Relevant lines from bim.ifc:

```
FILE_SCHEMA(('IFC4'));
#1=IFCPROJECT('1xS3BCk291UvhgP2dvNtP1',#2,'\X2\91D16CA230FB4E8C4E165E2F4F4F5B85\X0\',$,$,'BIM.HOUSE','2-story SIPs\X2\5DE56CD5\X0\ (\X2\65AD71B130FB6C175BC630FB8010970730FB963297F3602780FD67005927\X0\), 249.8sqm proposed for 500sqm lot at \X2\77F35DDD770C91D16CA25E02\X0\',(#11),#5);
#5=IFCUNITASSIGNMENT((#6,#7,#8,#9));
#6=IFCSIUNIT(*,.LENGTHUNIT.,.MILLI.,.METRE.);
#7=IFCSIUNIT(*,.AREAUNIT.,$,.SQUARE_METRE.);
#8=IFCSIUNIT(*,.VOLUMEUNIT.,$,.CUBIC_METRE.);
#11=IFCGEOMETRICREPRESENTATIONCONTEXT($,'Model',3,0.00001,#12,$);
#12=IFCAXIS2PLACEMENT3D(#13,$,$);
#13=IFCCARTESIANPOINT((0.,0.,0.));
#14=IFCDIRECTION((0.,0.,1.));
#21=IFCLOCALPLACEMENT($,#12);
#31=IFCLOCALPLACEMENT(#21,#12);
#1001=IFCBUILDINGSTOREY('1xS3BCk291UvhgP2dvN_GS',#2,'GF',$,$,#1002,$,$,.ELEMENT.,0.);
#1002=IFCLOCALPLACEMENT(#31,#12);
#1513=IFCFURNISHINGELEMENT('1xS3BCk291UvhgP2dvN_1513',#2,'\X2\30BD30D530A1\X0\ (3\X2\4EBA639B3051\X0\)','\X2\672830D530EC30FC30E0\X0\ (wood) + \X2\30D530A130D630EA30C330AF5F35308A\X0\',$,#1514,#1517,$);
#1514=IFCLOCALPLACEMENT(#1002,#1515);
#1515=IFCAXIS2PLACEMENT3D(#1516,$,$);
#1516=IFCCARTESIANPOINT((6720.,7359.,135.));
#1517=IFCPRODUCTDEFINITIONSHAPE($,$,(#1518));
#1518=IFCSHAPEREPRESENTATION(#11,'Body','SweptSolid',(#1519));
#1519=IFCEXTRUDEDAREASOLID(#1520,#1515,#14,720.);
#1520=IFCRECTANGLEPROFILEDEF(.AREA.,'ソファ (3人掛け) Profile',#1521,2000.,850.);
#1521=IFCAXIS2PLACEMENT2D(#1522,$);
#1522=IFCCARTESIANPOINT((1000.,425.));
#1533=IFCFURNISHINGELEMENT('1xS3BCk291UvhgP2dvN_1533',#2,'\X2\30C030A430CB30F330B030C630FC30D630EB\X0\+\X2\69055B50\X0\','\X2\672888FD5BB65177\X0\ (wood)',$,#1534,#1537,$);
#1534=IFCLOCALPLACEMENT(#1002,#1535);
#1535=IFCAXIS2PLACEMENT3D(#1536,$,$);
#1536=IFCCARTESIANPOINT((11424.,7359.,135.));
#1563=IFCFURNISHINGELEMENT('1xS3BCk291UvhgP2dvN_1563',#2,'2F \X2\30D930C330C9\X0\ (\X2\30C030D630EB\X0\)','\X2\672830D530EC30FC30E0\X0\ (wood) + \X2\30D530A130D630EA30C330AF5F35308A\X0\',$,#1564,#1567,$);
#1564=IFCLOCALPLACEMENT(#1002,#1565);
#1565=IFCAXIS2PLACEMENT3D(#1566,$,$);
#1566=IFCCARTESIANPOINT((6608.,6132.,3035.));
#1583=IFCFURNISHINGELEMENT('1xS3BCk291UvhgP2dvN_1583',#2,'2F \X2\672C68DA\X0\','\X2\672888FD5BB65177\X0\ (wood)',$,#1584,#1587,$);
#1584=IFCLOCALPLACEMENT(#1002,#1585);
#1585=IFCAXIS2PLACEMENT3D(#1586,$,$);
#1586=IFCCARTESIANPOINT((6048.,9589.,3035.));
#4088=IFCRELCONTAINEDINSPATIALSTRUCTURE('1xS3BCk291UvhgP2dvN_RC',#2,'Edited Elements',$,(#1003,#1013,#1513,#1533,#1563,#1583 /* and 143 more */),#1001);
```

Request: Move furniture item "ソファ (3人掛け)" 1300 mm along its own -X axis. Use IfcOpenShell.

```python
import ifcopenshell
import ifcopenshell.api.geometry
import ifcopenshell.util.placement

model = ifcopenshell.open("bim.ifc")

item = model.by_guid("1xS3BCk291UvhgP2dvN_1513")
matrix = ifcopenshell.util.placement.get_local_placement(item.ObjectPlacement)
matrix[:3, 3] -= matrix[:3, 0] * 1300.0
ifcopenshell.api.geometry.edit_object_placement(model, product=item, matrix=matrix, is_si=False)

print(ifcopenshell.util.placement.get_local_placement(item.ObjectPlacement).round(3) + 0.0)

model.write("bim_updated.ifc")
```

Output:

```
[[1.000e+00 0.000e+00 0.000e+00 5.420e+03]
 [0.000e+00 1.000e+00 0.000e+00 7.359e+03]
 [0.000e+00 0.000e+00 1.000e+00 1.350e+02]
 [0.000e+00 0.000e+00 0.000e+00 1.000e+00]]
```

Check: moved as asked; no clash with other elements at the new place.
